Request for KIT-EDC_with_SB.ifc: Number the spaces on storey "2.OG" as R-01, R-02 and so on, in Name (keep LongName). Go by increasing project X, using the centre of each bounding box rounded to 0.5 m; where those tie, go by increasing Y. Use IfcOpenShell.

First a look at what the model holds.

```python
import ifcopenshell
import ifcopenshell.util.element
import ifcopenshell.util.placement

model = ifcopenshell.open("KIT-EDC_with_SB.ifc")
print(model.schema)
storey = next(s for s in model.by_type("IfcBuildingStorey") if s.Name == "2.OG")
spaces = [e for e in ifcopenshell.util.element.get_decomposition(storey) if e.is_a("IfcSpace")]
for e in sorted(spaces, key=lambda e: e.id()):
    origin = ifcopenshell.util.placement.get_local_placement(e.ObjectPlacement)[:3, 3]
    print(e.id(), e.Name, e.LongName, origin.round(2) + 0.0, sep=" | ")
```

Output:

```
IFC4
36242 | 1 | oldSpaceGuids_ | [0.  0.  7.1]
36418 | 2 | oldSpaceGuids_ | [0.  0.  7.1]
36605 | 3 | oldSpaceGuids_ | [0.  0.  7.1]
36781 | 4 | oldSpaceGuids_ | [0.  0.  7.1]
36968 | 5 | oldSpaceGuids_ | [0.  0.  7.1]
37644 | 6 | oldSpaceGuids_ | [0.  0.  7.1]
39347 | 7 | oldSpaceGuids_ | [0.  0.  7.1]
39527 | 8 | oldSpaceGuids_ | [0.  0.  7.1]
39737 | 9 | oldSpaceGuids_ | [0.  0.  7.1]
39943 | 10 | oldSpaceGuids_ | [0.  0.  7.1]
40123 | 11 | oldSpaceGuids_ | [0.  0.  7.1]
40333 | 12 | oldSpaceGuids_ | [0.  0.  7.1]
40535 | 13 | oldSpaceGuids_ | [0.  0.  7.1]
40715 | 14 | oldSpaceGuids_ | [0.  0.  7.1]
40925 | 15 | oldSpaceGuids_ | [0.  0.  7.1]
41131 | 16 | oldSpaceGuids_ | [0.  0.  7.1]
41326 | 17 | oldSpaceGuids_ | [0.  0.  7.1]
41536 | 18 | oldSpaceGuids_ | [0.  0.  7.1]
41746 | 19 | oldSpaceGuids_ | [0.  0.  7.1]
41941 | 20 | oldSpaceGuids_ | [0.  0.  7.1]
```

```python
import ifcopenshell
import ifcopenshell.geom
import ifcopenshell.util.element
import ifcopenshell.util.shape

model = ifcopenshell.open("KIT-EDC_with_SB.ifc")
settings = ifcopenshell.geom.settings()
settings.set("use-world-coords", True)


def centre(element):
    shape = ifcopenshell.geom.create_shape(settings, element)
    return ifcopenshell.util.shape.get_bbox_centroid(shape.geometry)


storey = next(s for s in model.by_type("IfcBuildingStorey") if s.Name == "2.OG")
spaces = [e for e in ifcopenshell.util.element.get_decomposition(storey) if e.is_a("IfcSpace")]

# Insertion points can sit at a corner or the storey origin, so sort by the geometry (in metres).
centres = {e: centre(e) for e in spaces}
spaces.sort(key=lambda e: (round(centres[e][0] / 0.5), centres[e][1]))

for i, e in enumerate(spaces, start=1):
    number = f"R-{i:02d}"
    e.Name = number
    print(e.id(), number)

model.write("KIT-EDC_with_SB_v2.ifc")
```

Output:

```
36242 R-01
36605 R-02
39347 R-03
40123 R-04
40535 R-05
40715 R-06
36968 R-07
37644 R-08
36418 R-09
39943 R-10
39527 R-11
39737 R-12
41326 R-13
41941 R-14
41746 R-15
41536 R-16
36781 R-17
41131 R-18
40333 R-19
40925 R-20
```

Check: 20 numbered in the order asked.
